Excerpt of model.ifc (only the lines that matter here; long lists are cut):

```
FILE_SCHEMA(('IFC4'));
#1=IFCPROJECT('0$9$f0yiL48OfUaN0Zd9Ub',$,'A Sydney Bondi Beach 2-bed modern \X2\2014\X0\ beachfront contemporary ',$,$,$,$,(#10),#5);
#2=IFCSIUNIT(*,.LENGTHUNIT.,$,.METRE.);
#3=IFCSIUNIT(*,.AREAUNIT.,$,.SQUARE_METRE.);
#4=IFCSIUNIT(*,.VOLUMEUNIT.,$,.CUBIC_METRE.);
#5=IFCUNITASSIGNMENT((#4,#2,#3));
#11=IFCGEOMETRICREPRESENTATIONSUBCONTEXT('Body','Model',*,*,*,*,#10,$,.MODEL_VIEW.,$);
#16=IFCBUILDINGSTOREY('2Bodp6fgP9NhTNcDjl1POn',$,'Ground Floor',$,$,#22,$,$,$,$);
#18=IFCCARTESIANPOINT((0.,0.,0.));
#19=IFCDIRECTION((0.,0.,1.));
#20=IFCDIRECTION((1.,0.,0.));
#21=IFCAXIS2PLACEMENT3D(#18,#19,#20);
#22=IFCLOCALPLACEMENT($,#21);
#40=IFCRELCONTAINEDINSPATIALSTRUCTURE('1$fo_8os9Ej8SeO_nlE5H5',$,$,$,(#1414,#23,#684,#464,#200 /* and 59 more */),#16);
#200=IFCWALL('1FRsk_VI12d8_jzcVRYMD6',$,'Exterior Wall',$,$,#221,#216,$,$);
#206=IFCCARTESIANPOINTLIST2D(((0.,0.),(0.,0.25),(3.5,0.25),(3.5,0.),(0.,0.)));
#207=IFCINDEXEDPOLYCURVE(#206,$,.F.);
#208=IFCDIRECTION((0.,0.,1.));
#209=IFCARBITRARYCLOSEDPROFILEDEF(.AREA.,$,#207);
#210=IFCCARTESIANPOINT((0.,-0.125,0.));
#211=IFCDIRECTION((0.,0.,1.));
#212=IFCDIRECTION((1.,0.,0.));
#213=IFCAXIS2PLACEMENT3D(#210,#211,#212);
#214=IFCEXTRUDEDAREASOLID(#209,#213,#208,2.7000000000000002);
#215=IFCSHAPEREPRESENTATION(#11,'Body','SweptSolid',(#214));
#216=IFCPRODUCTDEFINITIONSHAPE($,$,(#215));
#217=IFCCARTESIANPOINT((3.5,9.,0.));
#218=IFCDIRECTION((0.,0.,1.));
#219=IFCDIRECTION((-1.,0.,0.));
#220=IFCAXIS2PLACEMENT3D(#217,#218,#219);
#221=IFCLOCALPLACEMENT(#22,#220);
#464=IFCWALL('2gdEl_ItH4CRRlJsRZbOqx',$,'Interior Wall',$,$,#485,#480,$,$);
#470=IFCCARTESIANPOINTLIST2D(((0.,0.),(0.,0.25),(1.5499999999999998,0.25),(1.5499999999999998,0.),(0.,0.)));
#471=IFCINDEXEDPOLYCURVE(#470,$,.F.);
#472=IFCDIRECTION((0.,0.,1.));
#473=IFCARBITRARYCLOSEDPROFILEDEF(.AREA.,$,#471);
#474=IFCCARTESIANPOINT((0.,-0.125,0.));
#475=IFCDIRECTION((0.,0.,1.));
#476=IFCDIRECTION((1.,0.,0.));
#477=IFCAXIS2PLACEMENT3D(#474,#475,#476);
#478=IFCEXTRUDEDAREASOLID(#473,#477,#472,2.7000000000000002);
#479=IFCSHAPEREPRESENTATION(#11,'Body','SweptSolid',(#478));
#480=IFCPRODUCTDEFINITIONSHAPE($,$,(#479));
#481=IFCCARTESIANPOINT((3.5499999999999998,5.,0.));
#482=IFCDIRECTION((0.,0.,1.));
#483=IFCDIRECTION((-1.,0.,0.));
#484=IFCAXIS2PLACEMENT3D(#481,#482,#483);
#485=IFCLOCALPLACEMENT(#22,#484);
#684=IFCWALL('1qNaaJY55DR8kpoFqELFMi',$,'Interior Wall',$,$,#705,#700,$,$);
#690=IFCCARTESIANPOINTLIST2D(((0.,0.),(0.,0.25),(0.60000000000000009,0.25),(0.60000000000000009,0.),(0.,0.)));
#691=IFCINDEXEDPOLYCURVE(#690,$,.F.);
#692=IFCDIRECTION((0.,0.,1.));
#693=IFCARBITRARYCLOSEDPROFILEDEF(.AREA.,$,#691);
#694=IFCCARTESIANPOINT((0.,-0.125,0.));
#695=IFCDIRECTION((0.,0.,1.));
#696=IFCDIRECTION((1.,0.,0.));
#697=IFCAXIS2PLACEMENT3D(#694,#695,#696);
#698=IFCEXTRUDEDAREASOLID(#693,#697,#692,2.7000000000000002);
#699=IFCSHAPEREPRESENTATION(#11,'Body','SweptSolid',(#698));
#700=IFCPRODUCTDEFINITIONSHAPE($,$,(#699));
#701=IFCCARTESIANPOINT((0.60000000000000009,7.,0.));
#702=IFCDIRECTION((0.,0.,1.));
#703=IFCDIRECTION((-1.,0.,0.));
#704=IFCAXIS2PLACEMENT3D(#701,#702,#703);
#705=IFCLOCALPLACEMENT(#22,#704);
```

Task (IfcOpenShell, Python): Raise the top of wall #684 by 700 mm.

```python
import ifcopenshell
import ifcopenshell.geom
import ifcopenshell.util.representation
import ifcopenshell.util.shape
import ifcopenshell.util.unit

model = ifcopenshell.open("model.ifc")
unit_scale = ifcopenshell.util.unit.calculate_unit_scale(model)
settings = ifcopenshell.geom.settings()


def volume(element):
    """Net volume in cubic metres, openings subtracted."""
    shape = ifcopenshell.geom.create_shape(settings, element)
    return ifcopenshell.util.shape.get_volume(shape.geometry)


wall = model.by_guid("1qNaaJY55DR8kpoFqELFMi")
before = volume(wall)

body = ifcopenshell.util.representation.get_representation(wall, "Model", "Body")
solid = body.Items[0]
old_height = solid.Depth
solid.Depth += 0.7 / unit_scale
after = volume(wall)

print(f"height {old_height:g} -> {solid.Depth:g}, volume {before:.3f} -> {after:.3f} m3")

model.write("model_edited.ifc")
```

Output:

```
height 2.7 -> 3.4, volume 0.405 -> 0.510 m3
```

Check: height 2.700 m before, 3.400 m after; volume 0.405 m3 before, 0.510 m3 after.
